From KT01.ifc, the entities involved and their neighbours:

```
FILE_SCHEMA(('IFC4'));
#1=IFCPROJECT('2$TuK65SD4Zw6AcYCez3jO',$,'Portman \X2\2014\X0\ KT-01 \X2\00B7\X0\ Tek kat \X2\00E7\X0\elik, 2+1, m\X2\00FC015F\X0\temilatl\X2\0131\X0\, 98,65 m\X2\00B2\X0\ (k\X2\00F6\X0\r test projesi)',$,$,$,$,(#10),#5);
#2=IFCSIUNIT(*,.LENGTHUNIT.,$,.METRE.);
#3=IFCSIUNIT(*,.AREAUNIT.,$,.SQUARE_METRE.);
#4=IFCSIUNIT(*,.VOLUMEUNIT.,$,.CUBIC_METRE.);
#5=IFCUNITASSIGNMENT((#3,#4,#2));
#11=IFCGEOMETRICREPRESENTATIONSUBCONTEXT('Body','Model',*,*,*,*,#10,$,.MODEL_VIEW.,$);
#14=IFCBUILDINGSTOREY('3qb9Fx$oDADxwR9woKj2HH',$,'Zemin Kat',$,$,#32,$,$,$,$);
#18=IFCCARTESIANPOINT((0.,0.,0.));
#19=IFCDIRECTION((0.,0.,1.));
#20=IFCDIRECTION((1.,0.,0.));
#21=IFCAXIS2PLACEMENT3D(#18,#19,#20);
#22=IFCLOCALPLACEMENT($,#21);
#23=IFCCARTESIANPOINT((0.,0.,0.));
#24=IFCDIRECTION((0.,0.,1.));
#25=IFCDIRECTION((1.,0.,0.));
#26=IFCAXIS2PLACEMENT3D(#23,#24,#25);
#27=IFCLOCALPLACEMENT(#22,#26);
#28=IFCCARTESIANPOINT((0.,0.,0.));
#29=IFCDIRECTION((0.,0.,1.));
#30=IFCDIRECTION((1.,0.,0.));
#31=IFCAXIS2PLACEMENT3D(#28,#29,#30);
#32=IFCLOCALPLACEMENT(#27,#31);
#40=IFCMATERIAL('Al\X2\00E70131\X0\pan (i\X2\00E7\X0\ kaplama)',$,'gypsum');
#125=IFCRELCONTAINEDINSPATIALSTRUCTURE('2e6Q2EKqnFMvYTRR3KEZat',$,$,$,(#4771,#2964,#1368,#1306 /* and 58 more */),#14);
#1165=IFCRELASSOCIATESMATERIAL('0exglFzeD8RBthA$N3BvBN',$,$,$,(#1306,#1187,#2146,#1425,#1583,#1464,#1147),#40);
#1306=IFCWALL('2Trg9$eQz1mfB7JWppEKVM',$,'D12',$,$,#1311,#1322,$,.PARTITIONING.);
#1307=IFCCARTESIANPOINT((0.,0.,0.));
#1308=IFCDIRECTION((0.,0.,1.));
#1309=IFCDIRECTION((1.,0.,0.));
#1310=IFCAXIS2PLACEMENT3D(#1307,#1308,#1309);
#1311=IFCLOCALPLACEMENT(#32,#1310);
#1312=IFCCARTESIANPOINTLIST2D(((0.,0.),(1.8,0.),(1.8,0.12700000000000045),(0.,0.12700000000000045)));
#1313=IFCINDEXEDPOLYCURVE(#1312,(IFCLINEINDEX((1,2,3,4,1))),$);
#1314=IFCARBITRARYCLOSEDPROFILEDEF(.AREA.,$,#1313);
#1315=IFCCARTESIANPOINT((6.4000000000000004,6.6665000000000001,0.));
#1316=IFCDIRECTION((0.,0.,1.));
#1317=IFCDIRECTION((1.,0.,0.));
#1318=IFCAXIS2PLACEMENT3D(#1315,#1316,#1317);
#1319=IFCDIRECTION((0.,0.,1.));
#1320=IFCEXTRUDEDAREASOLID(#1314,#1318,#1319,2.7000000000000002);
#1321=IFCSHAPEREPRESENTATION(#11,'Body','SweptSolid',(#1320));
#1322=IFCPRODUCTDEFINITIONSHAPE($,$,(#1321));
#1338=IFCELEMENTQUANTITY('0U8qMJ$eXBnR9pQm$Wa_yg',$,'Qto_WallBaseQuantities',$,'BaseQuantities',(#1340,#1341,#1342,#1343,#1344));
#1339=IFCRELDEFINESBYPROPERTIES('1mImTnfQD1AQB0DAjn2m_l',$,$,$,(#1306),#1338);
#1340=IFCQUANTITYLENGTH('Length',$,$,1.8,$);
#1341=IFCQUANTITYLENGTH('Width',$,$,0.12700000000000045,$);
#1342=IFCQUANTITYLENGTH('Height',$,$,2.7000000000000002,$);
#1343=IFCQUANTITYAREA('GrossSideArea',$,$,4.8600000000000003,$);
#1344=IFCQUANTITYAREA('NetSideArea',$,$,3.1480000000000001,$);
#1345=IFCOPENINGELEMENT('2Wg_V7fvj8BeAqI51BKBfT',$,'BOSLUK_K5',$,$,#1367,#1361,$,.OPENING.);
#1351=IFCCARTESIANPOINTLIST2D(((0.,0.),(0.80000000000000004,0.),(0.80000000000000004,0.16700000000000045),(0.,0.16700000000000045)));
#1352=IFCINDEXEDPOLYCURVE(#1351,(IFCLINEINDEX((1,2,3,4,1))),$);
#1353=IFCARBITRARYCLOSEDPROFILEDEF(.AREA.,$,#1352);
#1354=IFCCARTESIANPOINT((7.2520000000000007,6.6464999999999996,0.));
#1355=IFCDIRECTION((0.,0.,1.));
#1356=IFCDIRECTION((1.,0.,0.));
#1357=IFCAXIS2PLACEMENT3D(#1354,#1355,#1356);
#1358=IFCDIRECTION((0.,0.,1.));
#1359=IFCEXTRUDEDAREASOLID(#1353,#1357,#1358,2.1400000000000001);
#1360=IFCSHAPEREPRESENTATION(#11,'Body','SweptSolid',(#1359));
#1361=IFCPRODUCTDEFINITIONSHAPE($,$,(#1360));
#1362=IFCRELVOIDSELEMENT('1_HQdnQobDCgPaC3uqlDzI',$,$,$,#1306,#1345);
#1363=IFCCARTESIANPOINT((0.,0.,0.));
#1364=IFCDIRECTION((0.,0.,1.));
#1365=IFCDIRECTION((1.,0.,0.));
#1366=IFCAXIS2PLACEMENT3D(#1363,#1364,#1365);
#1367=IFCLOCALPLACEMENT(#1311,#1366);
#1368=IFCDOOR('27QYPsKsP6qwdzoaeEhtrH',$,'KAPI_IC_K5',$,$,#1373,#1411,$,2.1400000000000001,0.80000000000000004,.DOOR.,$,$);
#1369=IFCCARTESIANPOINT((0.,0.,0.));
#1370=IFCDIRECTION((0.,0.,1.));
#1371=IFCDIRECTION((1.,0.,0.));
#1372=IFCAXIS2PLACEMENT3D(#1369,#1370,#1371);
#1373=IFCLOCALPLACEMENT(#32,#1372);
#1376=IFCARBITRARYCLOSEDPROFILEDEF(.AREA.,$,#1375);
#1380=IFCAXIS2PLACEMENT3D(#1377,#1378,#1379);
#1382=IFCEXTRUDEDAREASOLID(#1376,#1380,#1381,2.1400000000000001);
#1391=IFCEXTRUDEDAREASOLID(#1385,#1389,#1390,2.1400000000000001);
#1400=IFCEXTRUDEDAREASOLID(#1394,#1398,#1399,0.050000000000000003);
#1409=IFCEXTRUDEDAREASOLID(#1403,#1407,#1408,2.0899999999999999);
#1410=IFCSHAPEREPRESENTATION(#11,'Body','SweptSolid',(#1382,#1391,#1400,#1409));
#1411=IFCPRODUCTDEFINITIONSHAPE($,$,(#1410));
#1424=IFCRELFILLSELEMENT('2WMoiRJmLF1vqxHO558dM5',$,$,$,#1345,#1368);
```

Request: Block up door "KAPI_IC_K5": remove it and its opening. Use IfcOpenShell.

```python
import ifcopenshell
import ifcopenshell.api.feature
import ifcopenshell.api.pset
import ifcopenshell.api.root
import ifcopenshell.geom
import ifcopenshell.util.element
import ifcopenshell.util.shape
import ifcopenshell.util.unit

model = ifcopenshell.open("KT01.ifc")
area_scale = ifcopenshell.util.unit.calculate_unit_scale(model, "AREAUNIT")
settings = ifcopenshell.geom.settings()


def volume(element):
    """Net volume in cubic metres, openings subtracted."""
    shape = ifcopenshell.geom.create_shape(settings, element)
    return ifcopenshell.util.shape.get_volume(shape.geometry)


door = model.by_guid("27QYPsKsP6qwdzoaeEhtrH")
opening = door.FillsVoids[0].RelatingOpeningElement
wall = opening.VoidsElements[0].RelatingBuildingElement
before = volume(wall)

ifcopenshell.api.root.remove_product(model, product=door)
ifcopenshell.api.feature.remove_feature(model, feature=opening)

after = volume(wall)
thickness = 0.127  # wall thickness in metres

# Update the wall's stored quantities.
qto = model.by_id(ifcopenshell.util.element.get_pset(wall, "Qto_WallBaseQuantities", should_inherit=False)["id"])
ifcopenshell.api.pset.edit_qto(model, qto=qto, properties={"NetSideArea": after / thickness / area_scale})

print(f"wall volume {before:.3f} -> {after:.3f} m3")

model.write("KT01_rev.ifc")
```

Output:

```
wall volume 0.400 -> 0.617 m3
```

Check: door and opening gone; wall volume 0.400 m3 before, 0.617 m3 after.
